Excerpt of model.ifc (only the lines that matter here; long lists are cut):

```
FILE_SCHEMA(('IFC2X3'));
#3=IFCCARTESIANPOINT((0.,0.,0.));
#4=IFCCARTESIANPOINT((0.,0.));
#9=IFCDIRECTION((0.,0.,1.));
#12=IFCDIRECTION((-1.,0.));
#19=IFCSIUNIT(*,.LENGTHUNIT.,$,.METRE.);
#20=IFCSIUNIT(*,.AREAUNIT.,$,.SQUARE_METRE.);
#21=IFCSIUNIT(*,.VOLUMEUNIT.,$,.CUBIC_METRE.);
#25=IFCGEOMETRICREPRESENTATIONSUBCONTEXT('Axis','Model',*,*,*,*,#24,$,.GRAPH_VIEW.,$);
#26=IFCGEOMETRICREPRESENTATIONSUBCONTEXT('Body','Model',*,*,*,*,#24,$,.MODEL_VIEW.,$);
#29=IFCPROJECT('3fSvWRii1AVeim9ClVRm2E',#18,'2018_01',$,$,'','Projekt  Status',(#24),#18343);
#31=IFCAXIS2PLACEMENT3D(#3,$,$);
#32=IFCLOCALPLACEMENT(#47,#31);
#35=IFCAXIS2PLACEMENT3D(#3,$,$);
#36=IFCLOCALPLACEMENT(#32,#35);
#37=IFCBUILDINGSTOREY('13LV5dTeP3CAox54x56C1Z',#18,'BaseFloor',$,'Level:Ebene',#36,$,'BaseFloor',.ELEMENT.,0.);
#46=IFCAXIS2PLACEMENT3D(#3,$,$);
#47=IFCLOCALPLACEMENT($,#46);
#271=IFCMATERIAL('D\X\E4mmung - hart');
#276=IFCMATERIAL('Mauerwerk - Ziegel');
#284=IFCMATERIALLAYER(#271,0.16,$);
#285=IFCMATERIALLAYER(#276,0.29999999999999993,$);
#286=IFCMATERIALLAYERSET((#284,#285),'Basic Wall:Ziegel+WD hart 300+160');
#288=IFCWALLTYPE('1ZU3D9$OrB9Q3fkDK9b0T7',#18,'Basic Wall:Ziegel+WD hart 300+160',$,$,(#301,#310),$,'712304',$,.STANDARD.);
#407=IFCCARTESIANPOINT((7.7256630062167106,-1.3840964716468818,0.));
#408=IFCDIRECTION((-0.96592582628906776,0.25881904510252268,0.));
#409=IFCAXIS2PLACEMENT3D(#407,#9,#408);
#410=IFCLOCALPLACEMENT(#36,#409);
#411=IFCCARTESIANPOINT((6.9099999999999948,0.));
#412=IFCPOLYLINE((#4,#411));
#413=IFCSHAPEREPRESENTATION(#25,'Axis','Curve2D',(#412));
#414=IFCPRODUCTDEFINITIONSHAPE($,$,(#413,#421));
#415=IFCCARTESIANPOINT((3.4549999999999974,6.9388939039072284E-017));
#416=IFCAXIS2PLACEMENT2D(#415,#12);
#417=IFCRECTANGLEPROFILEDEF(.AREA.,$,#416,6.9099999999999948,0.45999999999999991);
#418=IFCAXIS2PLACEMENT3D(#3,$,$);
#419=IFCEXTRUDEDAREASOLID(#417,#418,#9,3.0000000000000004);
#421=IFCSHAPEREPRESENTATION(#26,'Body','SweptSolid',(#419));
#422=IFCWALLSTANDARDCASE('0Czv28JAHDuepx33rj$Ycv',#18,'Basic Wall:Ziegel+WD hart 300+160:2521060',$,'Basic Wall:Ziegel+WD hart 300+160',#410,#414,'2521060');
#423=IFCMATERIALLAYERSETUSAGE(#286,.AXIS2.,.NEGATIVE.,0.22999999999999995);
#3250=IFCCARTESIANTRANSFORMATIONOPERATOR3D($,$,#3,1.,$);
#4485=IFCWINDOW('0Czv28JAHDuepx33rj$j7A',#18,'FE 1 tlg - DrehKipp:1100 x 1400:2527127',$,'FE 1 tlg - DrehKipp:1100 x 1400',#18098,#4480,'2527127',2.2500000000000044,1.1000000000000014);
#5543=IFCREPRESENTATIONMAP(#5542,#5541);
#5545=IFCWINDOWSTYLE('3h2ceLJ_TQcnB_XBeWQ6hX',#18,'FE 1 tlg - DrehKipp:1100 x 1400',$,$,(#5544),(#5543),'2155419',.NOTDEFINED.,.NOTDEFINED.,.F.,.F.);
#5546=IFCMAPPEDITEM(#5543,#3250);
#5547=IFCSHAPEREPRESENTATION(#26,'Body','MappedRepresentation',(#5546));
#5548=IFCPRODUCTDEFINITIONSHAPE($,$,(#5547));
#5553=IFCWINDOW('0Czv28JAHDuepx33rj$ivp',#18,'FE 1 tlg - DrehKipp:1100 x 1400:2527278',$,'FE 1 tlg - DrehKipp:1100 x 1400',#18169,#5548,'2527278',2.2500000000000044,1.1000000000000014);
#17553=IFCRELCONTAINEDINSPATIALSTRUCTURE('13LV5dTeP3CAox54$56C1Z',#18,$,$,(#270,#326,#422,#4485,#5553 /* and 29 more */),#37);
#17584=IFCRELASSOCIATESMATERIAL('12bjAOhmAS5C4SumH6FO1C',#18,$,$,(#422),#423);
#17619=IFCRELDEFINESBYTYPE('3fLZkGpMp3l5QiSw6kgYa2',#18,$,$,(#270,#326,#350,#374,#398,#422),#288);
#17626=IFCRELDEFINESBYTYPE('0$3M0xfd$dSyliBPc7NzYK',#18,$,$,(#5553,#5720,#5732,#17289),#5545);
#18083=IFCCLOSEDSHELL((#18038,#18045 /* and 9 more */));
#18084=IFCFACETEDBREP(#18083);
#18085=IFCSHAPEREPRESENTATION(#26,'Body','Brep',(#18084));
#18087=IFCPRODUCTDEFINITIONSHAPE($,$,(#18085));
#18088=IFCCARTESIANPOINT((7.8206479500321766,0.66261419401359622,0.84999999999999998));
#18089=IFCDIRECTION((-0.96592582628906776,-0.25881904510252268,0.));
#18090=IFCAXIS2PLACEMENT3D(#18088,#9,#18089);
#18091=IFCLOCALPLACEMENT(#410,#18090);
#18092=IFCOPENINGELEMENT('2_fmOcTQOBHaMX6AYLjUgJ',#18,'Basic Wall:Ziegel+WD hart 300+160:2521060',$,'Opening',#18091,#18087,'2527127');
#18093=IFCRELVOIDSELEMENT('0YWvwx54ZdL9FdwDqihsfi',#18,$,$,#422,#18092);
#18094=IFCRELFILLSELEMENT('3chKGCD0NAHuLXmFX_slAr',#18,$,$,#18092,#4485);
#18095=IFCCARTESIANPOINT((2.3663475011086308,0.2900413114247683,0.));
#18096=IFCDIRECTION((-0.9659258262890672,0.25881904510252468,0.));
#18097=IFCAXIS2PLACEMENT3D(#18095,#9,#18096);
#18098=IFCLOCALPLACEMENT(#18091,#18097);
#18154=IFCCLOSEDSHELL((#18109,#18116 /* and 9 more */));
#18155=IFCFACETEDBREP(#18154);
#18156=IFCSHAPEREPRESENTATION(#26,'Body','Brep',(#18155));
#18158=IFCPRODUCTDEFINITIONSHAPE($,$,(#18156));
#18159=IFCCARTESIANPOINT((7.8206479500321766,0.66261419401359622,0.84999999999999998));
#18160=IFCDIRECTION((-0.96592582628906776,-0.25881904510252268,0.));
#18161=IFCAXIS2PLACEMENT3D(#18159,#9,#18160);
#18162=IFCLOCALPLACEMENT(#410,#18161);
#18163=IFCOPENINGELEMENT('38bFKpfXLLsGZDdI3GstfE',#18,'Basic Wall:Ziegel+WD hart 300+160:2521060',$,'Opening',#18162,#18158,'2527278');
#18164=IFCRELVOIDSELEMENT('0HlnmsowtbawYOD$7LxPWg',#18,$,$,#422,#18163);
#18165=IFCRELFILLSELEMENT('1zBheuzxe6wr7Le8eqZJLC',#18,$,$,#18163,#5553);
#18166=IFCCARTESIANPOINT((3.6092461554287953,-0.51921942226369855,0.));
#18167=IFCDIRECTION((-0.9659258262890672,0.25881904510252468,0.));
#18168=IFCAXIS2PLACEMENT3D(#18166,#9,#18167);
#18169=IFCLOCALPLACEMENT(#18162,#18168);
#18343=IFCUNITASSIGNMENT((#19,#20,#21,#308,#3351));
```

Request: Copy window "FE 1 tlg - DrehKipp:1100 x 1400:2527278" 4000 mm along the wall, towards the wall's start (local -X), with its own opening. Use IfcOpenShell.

```python
import ifcopenshell
import ifcopenshell.api.feature
import ifcopenshell.api.geometry
import ifcopenshell.api.root
import ifcopenshell.geom
import ifcopenshell.util.element
import ifcopenshell.util.placement
import ifcopenshell.util.shape

model = ifcopenshell.open("model.ifc")
settings = ifcopenshell.geom.settings()


def volume(element):
    """Net volume in cubic metres, openings subtracted."""
    shape = ifcopenshell.geom.create_shape(settings, element)
    return ifcopenshell.util.shape.get_volume(shape.geometry)


def reuse_history(source, copy):
    """copy_class also copies each property set's owner history, people and application; keep the originals."""
    for rel in copy.IsDefinedBy:
        if rel.is_a("IfcRelDefinesByProperties") and (history := rel.RelatingPropertyDefinition.OwnerHistory):
            rel.RelatingPropertyDefinition.OwnerHistory = source.OwnerHistory
            ifcopenshell.util.element.remove_deep2(model, history)


window = model.by_guid("0Czv28JAHDuepx33rj$ivp")
opening = window.FillsVoids[0].RelatingOpeningElement
wall = opening.VoidsElements[0].RelatingBuildingElement
before = volume(wall)
shift = ifcopenshell.util.placement.get_local_placement(wall.ObjectPlacement)[:3, 0] * -4.0

# copy_class copies the void relationship, type, container and properties, but no geometry.
new_opening = ifcopenshell.api.root.copy_class(model, product=opening)
new_opening.Representation = ifcopenshell.util.element.copy_deep(
    model, opening.Representation, exclude=["IfcGeometricRepresentationContext", "IfcRepresentationMap"]
)
new_opening.Name = "Basic Wall:Ziegel+WD hart 300+160"
new_opening.Tag = None
new_window = ifcopenshell.api.root.copy_class(model, product=window)
new_window.Representation = ifcopenshell.util.element.copy_deep(
    model, window.Representation, exclude=["IfcGeometricRepresentationContext", "IfcRepresentationMap"]
)
new_window.Name = "FE 1 tlg - DrehKipp:1100 x 1400"
new_window.Tag = None
reuse_history(window, new_window)
fills = ifcopenshell.api.feature.add_filling(model, opening=new_opening, element=new_window)
fills.OwnerHistory = new_window.OwnerHistory  # required in IFC2X3

for old, new in ((opening, new_opening), (window, new_window)):
    matrix = ifcopenshell.util.placement.get_local_placement(old.ObjectPlacement)
    matrix[:3, 3] += shift
    ifcopenshell.api.geometry.edit_object_placement(model, product=new, matrix=matrix, is_si=False)

after = volume(wall)

print(f"wall volume {before:.3f} -> {after:.3f} m3")

model.write("model_rev.ifc")
```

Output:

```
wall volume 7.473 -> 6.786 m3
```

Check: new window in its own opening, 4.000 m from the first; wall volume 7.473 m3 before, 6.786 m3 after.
